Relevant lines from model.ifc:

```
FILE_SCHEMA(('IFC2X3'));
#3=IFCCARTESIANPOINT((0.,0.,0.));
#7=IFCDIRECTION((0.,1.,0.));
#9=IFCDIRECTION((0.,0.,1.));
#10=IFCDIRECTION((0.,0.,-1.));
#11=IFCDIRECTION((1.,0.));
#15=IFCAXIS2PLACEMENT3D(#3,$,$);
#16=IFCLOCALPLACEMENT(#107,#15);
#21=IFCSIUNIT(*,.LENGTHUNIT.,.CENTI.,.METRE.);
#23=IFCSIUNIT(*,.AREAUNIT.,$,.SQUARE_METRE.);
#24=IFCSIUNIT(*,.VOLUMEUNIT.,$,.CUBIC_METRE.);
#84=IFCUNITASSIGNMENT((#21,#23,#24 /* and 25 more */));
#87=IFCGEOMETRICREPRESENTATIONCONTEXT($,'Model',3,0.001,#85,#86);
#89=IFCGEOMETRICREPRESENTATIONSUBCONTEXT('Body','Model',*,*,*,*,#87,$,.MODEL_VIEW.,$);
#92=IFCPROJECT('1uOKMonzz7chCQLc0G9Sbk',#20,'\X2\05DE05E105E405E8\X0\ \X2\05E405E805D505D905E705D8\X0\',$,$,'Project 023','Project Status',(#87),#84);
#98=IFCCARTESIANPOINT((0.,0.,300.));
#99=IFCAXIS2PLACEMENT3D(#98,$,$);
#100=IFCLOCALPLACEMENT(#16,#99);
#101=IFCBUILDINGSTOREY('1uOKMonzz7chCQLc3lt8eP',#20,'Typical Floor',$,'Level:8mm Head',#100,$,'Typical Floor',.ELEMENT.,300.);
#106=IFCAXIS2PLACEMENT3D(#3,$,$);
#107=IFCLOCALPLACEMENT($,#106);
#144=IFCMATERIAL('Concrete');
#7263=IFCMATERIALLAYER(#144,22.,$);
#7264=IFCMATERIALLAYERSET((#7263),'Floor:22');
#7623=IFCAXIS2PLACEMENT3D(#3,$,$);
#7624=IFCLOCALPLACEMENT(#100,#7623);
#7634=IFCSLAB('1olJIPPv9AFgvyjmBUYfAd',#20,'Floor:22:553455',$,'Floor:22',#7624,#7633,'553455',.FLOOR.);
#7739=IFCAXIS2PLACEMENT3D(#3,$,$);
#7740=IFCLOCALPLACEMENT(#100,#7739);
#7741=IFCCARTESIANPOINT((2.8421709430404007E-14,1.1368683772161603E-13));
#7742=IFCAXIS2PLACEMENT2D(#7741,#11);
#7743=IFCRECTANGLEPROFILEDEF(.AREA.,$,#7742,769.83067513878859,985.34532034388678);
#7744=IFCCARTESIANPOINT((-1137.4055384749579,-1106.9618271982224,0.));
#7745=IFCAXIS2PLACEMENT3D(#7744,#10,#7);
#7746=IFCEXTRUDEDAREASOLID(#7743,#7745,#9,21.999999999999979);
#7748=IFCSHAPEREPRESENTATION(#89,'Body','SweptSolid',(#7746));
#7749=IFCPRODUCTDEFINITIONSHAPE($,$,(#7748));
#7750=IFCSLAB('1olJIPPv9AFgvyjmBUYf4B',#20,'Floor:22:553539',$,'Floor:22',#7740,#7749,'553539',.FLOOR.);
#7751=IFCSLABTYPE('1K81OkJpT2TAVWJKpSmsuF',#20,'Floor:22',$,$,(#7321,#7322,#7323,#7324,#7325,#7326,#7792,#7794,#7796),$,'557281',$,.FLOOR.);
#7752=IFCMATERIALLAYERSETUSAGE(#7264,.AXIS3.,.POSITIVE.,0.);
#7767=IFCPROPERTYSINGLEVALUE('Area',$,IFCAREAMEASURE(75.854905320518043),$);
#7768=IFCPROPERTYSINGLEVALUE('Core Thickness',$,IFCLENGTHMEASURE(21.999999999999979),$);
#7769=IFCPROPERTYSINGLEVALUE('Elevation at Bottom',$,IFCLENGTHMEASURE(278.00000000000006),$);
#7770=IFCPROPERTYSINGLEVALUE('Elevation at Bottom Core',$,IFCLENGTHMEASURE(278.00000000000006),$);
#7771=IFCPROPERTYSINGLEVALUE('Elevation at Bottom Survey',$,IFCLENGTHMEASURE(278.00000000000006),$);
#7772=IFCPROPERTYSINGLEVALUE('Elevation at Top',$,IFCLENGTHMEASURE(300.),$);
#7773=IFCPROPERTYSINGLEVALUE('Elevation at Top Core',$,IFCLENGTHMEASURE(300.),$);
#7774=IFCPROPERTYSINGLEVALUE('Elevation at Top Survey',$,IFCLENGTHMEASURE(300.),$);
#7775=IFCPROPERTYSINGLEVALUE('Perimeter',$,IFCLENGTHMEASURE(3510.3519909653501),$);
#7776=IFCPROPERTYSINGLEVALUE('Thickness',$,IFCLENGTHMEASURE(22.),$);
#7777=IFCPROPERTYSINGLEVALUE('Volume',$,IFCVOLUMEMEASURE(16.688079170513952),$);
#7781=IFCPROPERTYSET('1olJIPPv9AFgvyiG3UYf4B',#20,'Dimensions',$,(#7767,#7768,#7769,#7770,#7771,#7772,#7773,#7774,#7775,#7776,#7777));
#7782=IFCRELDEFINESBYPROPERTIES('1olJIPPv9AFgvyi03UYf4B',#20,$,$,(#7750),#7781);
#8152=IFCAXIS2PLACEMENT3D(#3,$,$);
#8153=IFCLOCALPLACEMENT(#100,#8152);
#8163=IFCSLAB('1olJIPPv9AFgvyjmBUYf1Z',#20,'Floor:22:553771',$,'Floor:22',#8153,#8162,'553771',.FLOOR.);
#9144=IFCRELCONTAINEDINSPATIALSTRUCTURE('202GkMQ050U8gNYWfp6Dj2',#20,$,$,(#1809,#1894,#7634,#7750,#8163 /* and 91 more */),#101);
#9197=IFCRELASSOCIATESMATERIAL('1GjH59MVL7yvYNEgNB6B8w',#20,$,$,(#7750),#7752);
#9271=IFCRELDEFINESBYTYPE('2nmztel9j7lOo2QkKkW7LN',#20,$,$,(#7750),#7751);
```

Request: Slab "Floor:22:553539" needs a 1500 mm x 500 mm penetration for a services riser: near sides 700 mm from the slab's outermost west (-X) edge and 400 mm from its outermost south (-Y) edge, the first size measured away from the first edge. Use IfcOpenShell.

```python
import numpy as np
import ifcopenshell
import ifcopenshell.api.feature
import ifcopenshell.api.geometry
import ifcopenshell.api.pset
import ifcopenshell.api.root
import ifcopenshell.geom
import ifcopenshell.util.element
import ifcopenshell.util.placement
import ifcopenshell.util.representation
import ifcopenshell.util.shape
import ifcopenshell.util.unit

model = ifcopenshell.open("model.ifc")
unit_scale = ifcopenshell.util.unit.calculate_unit_scale(model)
area_scale = ifcopenshell.util.unit.calculate_unit_scale(model, "AREAUNIT")
volume_scale = ifcopenshell.util.unit.calculate_unit_scale(model, "VOLUMEUNIT")
settings = ifcopenshell.geom.settings()


def volume(element):
    """Net volume in cubic metres, openings subtracted."""
    shape = ifcopenshell.geom.create_shape(settings, element)
    return ifcopenshell.util.shape.get_volume(shape.geometry)


slab = model.by_id(7750)
before = volume(slab)

# Extent in the slab's own axes, in metres. The edges named are its -X and -Y sides.
slab_shape = ifcopenshell.geom.create_shape(settings, slab)
vertices = ifcopenshell.util.shape.get_vertices(slab_shape.geometry)
x_min, y_min, bottom = vertices.min(axis=0)
top = vertices[:, 2].max()

opening = ifcopenshell.api.root.create_entity(model, ifc_class="IfcOpeningElement", name="Services riser opening")
context = ifcopenshell.util.representation.get_context(model, "Model", "Body", "MODEL_VIEW")
width, depth = 1.5, 0.5
outline = [(0.0, 0.0), (width, 0.0), (width, depth), (0.0, depth), (0.0, 0.0)]
# Overshoot both faces by 50 mm so the cut is clean.
shape = ifcopenshell.api.geometry.add_slab_representation(
    model, context=context, depth=top - bottom + 0.1, polyline=outline
)
ifcopenshell.api.geometry.assign_representation(model, product=opening, representation=shape)

matrix = ifcopenshell.util.placement.get_local_placement(slab.ObjectPlacement)
matrix[:, 3] = matrix @ np.append(np.array([x_min + 0.7, y_min + 0.4, bottom - 0.05]) / unit_scale, 1.0)
ifcopenshell.api.geometry.edit_object_placement(model, product=opening, matrix=matrix, is_si=False)
ifcopenshell.api.feature.add_feature(model, feature=opening, element=slab)

after = volume(slab)

# Update the slab's stored quantities.
pset = model.by_id(ifcopenshell.util.element.get_pset(slab, "Dimensions", should_inherit=False)["id"])
ifcopenshell.api.pset.edit_pset(model, pset=pset, properties={
    "Area": model.create_entity("IfcAreaMeasure", after / (top - bottom) / area_scale),
    "Volume": model.create_entity("IfcVolumeMeasure", after / volume_scale),
})

print(f"slab volume {before:.3f} -> {after:.3f} m3")

model.write("model_rev.ifc")
```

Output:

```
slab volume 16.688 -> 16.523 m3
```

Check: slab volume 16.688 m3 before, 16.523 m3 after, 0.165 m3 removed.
